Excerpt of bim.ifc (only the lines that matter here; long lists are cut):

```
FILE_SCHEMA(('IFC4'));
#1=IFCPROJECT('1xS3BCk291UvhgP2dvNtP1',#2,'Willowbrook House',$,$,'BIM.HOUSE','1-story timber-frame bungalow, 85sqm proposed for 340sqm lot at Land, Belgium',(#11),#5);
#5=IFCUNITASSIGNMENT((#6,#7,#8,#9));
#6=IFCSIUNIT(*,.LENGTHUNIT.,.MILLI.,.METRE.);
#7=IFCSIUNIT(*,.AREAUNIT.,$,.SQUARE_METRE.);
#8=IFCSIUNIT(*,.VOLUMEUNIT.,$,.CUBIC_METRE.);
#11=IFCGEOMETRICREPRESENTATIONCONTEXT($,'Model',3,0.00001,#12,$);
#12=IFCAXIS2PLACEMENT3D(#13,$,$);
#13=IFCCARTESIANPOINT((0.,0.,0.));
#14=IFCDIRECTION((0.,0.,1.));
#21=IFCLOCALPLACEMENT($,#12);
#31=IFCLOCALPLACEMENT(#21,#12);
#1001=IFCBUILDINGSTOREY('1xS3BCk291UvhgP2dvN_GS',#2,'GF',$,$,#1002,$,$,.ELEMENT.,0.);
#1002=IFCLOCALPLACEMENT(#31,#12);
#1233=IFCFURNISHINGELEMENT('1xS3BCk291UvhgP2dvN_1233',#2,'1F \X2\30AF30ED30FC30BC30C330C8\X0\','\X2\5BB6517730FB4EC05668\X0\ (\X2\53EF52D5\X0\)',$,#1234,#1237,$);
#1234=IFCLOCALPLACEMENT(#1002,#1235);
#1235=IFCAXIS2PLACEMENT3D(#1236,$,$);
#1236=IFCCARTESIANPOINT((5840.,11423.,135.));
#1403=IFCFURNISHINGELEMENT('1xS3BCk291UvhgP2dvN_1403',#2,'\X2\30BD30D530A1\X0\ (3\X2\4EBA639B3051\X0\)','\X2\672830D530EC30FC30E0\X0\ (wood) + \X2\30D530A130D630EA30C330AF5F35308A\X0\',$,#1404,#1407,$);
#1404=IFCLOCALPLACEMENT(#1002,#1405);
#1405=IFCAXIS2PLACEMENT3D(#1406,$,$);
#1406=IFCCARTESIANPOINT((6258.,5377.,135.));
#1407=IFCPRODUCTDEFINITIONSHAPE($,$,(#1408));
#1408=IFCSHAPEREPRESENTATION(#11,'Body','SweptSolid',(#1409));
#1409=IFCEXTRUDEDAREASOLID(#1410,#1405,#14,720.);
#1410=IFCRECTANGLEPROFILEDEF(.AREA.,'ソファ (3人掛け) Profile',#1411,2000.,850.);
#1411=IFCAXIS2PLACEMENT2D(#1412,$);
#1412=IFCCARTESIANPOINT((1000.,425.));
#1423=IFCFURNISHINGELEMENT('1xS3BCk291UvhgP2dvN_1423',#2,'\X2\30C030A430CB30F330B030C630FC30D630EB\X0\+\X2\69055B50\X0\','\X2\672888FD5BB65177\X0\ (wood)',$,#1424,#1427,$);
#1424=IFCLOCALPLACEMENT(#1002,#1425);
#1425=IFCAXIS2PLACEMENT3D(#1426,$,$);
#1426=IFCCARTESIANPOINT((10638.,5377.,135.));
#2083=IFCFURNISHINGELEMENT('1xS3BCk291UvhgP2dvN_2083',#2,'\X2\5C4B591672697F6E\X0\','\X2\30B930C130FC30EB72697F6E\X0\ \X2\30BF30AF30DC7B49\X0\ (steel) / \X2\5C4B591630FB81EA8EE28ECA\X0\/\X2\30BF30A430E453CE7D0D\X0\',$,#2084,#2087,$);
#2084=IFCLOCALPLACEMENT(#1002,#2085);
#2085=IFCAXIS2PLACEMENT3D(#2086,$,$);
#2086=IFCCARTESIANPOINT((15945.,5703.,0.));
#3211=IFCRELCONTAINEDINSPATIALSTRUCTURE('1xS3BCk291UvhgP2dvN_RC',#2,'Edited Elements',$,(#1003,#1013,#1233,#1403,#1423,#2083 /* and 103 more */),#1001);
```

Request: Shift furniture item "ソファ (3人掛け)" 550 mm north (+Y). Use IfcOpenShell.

```python
import ifcopenshell
import ifcopenshell.api.geometry
import ifcopenshell.util.placement
import ifcopenshell.util.unit

model = ifcopenshell.open("bim.ifc")
unit_scale = ifcopenshell.util.unit.calculate_unit_scale(model)

item = model.by_guid("1xS3BCk291UvhgP2dvN_1403")
matrix = ifcopenshell.util.placement.get_local_placement(item.ObjectPlacement)
matrix[1, 3] += 0.55 / unit_scale
ifcopenshell.api.geometry.edit_object_placement(model, product=item, matrix=matrix, is_si=False)

print(ifcopenshell.util.placement.get_local_placement(item.ObjectPlacement).round(3) + 0.0)

model.write("bim_rev.ifc")
```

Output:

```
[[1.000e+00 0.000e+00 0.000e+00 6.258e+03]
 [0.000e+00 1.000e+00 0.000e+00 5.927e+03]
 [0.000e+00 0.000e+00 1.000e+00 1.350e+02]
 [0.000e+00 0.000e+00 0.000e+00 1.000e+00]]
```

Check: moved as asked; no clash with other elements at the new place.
